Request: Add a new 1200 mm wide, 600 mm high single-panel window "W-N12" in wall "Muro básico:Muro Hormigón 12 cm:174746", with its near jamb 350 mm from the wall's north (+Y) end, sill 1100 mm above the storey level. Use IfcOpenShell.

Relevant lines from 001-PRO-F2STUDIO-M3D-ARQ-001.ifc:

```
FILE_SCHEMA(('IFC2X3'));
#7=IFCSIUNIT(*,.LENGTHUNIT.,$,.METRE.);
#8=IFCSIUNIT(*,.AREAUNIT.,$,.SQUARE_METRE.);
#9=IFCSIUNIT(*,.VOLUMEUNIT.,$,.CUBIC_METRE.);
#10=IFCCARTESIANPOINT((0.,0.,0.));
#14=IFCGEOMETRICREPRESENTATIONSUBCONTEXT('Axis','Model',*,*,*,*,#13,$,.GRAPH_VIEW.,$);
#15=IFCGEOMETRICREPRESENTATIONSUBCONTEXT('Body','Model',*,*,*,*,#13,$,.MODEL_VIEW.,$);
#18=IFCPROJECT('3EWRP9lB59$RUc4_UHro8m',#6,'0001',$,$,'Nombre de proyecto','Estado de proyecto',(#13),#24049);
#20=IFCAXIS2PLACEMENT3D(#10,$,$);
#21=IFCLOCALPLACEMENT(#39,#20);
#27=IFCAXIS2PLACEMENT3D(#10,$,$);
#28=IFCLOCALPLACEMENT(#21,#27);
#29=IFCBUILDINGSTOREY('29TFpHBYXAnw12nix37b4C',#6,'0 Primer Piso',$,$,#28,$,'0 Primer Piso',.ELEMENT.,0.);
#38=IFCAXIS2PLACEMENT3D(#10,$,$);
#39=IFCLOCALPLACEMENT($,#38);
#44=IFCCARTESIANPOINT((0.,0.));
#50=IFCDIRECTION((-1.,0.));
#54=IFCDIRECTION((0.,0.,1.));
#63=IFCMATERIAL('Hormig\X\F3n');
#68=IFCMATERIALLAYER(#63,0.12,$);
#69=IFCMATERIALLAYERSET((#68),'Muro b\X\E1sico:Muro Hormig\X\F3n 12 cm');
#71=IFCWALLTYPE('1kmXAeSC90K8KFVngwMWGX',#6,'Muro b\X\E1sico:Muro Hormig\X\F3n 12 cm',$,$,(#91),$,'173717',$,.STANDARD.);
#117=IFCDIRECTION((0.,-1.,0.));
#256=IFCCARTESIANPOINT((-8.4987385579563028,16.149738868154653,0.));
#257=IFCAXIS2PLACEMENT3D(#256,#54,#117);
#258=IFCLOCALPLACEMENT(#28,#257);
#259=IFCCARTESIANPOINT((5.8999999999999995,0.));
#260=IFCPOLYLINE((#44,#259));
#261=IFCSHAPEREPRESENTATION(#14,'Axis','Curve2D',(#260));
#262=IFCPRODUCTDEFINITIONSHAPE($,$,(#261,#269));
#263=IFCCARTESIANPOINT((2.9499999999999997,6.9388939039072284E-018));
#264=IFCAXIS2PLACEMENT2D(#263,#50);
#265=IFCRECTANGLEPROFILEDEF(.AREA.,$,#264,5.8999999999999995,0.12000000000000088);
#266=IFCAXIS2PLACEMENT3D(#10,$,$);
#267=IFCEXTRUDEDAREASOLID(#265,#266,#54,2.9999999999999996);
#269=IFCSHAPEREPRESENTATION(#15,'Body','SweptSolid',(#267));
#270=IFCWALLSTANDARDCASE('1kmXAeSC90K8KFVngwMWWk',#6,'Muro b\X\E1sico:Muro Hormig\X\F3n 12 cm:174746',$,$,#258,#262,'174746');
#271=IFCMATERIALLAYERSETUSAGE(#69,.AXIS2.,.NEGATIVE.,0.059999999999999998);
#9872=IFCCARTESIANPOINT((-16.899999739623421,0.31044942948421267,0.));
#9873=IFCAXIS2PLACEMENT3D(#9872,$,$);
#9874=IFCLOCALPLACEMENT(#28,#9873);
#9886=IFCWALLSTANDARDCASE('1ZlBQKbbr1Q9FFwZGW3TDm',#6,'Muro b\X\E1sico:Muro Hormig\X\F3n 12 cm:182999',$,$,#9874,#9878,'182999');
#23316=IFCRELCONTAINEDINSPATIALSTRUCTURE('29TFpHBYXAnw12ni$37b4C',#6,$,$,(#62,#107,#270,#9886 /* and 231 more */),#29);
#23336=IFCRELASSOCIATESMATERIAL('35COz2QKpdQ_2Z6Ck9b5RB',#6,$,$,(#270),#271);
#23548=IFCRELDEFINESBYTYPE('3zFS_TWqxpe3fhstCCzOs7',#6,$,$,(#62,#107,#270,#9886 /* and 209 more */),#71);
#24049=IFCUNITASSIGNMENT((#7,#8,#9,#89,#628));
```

```python
import numpy as np
import ifcopenshell
import ifcopenshell.api.feature
import ifcopenshell.api.geometry
import ifcopenshell.api.root
import ifcopenshell.api.spatial
import ifcopenshell.api.type
import ifcopenshell.geom
import ifcopenshell.util.element
import ifcopenshell.util.placement
import ifcopenshell.util.representation
import ifcopenshell.util.shape
import ifcopenshell.util.unit

model = ifcopenshell.open("001-PRO-F2STUDIO-M3D-ARQ-001.ifc")
unit_scale = ifcopenshell.util.unit.calculate_unit_scale(model)
settings = ifcopenshell.geom.settings()


def volume(element):
    """Net volume in cubic metres, openings subtracted."""
    shape = ifcopenshell.geom.create_shape(settings, element)
    return ifcopenshell.util.shape.get_volume(shape.geometry)


wall = model.by_guid("1kmXAeSC90K8KFVngwMWWk")
storey = ifcopenshell.util.element.get_container(wall, ifc_class="IfcBuildingStorey")
context = ifcopenshell.util.representation.get_context(model, "Model", "Body", "MODEL_VIEW")
before = volume(wall)

width, height, from_end, sill = 1.2, 0.6, 0.35, 1.1  # metres

# The wall runs along its own X axis, and the end named is its -X end.
wall_shape = ifcopenshell.geom.create_shape(settings, wall)
x, y, z = ifcopenshell.util.shape.get_vertices(wall_shape.geometry).T
start = x.min() + from_end
face, thickness = float(y.min()), float(y.max() - y.min())
wall_matrix = ifcopenshell.util.placement.get_local_placement(wall.ObjectPlacement)
level = ifcopenshell.util.placement.get_local_placement(storey.ObjectPlacement)[2, 3]


def in_wall(x, y):
    """Placement at x, y metres in the wall's axes, at sill height."""
    matrix = wall_matrix.copy()
    matrix[:, 3] = wall_matrix @ np.array([x / unit_scale, y / unit_scale, 0.0, 1.0])
    matrix[2, 3] = level + sill / unit_scale
    return matrix


# Opening: a box that overshoots both wall faces by 50 mm.
opening = ifcopenshell.api.root.create_entity(model, ifc_class="IfcOpeningElement")
box = ifcopenshell.api.geometry.add_wall_representation(
    model, context=context, length=width, height=height, thickness=thickness + 0.1
)
ifcopenshell.api.geometry.assign_representation(model, product=opening, representation=box)
ifcopenshell.api.geometry.edit_object_placement(model, product=opening, matrix=in_wall(start, face - 0.05), is_si=False)
ifcopenshell.api.feature.add_feature(model, feature=opening, element=wall)

window = ifcopenshell.api.root.create_entity(model, ifc_class="IfcWindow", name="W-N12")
window.OverallWidth, window.OverallHeight = width / unit_scale, height / unit_scale
body = ifcopenshell.api.geometry.add_window_representation(
    model,
    context=context,
    overall_width=window.OverallWidth,
    overall_height=window.OverallHeight,
    partition_type="SINGLE_PANEL",
)
ifcopenshell.api.geometry.assign_representation(model, product=window, representation=body)
ifcopenshell.api.spatial.assign_container(model, products=[window], relating_structure=storey)
fills = ifcopenshell.api.feature.add_filling(model, opening=opening, element=window)
fills.OwnerHistory = window.OwnerHistory  # required in IFC2X3

# IFC2X3 keeps the operation on the window style.
style = ifcopenshell.api.root.create_entity(model, ifc_class="IfcWindowStyle", name="W-N12")
style.OperationType, style.ConstructionType = "SINGLE_PANEL", "NOTDEFINED"
style.ParameterTakesPrecedence = style.Sizeable = False
ifcopenshell.api.type.assign_type(model, related_objects=[window], relating_type=style)

# Centre the window in the wall's thickness.
ifcopenshell.api.geometry.edit_object_placement(model, product=window, matrix=in_wall(start, face), is_si=False)
window_shape = ifcopenshell.geom.create_shape(settings, window)
depth = ifcopenshell.util.shape.get_vertices(window_shape.geometry)[:, 1]
offset = face + thickness / 2 - (depth.min() + depth.max()) / 2
ifcopenshell.api.geometry.edit_object_placement(model, product=window, matrix=in_wall(start, offset), is_si=False)

after = volume(wall)

print(f"wall volume {before:.3f} -> {after:.3f} m3")

model.write("001-PRO-F2STUDIO-M3D-ARQ-001_v2.ifc")
```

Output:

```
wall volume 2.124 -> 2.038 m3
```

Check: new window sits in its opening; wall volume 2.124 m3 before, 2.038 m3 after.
